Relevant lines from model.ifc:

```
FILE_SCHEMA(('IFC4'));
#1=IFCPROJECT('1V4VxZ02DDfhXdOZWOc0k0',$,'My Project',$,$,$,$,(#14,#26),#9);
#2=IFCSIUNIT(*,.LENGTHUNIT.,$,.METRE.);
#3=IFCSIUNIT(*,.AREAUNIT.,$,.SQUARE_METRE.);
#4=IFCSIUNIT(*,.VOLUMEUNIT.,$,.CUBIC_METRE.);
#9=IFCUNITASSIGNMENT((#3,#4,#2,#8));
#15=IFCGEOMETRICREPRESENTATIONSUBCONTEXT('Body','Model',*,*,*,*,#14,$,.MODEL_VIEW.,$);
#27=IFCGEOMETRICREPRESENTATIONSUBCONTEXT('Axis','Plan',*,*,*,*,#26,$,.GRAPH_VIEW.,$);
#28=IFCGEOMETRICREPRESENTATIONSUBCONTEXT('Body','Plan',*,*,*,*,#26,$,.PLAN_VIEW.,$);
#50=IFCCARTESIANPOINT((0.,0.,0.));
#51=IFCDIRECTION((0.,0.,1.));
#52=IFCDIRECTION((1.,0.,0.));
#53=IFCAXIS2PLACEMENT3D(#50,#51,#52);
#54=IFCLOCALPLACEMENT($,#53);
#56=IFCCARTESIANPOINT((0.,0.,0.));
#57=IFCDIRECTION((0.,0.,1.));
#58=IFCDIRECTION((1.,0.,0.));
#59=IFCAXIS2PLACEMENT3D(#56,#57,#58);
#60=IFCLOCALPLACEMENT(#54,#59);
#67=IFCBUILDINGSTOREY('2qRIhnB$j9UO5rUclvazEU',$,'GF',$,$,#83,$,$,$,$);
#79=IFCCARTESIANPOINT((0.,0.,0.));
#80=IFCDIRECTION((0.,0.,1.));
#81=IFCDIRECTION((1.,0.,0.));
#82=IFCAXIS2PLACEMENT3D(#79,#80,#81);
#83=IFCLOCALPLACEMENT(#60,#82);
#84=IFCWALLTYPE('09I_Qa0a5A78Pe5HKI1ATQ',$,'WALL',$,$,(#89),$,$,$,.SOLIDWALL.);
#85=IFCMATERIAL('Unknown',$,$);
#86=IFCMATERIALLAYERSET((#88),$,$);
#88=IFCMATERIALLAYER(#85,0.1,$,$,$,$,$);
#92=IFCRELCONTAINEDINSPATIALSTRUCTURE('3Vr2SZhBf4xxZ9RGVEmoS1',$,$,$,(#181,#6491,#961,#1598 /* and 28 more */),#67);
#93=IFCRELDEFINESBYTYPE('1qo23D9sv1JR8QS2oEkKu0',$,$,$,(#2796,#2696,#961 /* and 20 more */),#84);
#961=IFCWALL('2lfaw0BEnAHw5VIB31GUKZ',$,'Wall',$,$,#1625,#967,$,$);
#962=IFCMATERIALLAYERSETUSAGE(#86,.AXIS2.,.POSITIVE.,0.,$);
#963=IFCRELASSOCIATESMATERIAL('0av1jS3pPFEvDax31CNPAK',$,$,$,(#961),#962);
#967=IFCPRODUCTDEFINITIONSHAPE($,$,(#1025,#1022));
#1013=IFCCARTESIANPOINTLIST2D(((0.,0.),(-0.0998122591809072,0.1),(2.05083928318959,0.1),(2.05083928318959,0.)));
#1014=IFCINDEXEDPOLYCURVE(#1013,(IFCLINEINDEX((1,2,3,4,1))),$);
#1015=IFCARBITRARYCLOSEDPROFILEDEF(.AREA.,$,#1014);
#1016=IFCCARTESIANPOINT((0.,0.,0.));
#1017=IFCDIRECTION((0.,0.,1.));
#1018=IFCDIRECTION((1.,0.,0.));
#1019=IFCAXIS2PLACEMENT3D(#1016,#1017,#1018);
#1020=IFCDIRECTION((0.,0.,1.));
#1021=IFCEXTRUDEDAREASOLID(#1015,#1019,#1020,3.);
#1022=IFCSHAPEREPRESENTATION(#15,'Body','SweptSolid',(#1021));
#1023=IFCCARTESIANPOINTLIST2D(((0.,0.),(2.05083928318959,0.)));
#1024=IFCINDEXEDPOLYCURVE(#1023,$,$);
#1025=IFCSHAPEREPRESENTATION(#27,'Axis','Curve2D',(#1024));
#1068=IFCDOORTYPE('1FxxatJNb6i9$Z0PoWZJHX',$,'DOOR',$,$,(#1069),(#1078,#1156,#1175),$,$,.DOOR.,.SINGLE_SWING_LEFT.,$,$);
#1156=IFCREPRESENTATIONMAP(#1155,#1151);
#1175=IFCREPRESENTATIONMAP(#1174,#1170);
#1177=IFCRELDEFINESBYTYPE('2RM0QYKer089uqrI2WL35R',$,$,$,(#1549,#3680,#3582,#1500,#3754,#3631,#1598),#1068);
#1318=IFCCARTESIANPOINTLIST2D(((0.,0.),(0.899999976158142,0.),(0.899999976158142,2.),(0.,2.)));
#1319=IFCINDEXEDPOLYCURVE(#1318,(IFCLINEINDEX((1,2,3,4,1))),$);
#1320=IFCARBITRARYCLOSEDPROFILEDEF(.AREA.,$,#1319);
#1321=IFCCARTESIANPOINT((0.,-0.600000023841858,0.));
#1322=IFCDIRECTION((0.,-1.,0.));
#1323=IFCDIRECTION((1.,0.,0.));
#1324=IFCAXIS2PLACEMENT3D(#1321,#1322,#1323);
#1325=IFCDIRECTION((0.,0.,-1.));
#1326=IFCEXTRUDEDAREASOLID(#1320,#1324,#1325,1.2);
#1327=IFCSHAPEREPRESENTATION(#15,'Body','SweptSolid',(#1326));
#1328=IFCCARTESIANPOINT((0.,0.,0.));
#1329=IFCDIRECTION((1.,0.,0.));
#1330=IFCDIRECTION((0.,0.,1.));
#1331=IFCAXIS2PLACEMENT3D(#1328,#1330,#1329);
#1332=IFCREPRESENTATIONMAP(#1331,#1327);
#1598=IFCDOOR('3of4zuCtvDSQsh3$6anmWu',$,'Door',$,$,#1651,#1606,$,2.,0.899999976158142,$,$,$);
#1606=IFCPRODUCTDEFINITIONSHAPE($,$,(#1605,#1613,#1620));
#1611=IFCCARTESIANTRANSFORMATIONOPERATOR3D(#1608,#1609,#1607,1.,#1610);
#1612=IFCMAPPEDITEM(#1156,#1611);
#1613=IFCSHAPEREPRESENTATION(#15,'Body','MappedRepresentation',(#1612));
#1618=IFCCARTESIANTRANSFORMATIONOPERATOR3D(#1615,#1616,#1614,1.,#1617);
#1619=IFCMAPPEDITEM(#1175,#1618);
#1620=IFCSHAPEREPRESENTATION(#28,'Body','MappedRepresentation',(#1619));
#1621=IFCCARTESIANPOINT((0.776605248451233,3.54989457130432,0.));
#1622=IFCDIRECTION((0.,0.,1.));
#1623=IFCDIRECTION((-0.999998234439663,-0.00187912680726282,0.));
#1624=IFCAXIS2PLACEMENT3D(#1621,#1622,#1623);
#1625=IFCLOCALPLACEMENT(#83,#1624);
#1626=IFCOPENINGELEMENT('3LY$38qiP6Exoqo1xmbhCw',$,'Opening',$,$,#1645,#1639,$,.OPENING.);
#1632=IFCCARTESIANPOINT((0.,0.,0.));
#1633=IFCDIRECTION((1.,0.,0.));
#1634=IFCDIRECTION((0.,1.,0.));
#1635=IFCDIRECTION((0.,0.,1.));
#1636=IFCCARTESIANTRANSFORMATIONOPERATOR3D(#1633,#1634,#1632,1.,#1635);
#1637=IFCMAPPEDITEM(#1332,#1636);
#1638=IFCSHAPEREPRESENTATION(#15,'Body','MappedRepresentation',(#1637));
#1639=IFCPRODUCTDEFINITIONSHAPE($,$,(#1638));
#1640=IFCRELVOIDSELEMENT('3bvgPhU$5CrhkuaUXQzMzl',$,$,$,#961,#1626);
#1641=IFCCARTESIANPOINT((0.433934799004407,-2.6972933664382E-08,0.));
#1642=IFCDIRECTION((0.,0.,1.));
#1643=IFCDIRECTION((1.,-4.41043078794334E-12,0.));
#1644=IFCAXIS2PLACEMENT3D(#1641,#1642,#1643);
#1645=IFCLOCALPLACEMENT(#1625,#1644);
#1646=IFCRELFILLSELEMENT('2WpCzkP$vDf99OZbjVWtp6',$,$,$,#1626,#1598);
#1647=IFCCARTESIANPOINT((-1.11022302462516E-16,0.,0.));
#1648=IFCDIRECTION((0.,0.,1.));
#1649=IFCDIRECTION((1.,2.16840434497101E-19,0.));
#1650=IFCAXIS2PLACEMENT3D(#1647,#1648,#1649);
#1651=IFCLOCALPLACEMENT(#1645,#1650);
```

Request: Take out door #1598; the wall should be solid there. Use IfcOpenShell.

```python
import ifcopenshell
import ifcopenshell.api.feature
import ifcopenshell.api.root
import ifcopenshell.geom
import ifcopenshell.util.shape

model = ifcopenshell.open("model.ifc")
settings = ifcopenshell.geom.settings()


def volume(element):
    """Net volume in cubic metres, openings subtracted."""
    shape = ifcopenshell.geom.create_shape(settings, element)
    return ifcopenshell.util.shape.get_volume(shape.geometry)


door = model.by_guid("3of4zuCtvDSQsh3$6anmWu")
opening = door.FillsVoids[0].RelatingOpeningElement
wall = opening.VoidsElements[0].RelatingBuildingElement
before = volume(wall)

ifcopenshell.api.root.remove_product(model, product=door)
ifcopenshell.api.feature.remove_feature(model, feature=opening)

after = volume(wall)

print(f"wall volume {before:.3f} -> {after:.3f} m3")

model.write("model_rev.ifc")
```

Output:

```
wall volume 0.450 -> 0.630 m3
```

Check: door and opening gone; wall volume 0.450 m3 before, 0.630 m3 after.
